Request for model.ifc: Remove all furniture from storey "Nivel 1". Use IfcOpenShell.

First a look at what the model holds.

```python
import ifcopenshell
import ifcopenshell.util.element

model = ifcopenshell.open("model.ifc")
print(model.schema)
storey = next(s for s in model.by_type("IfcBuildingStorey") if s.Name == "Nivel 1")
furniture = [e for e in ifcopenshell.util.element.get_decomposition(storey) if e.is_a("IfcFurnishingElement")]
seen = {}
for e in furniture:
    element_type = ifcopenshell.util.element.get_type(e)
    name = element_type.Name if element_type not in (None, e) else None
    seen[name] = seen.get(name, 0) + 1
for name, count in sorted(seen.items(), key=str):
    print(count, "x", name)
```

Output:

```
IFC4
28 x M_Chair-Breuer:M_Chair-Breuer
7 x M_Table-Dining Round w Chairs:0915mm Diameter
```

```python
import ifcopenshell
import ifcopenshell.api.root
import ifcopenshell.util.element

model = ifcopenshell.open("model.ifc")

storey = next(s for s in model.by_type("IfcBuildingStorey") if s.Name == "Nivel 1")
furniture = [e for e in ifcopenshell.util.element.get_decomposition(storey) if e.is_a("IfcFurnishingElement")]

for e in furniture:
    ifcopenshell.api.root.remove_product(model, product=e)
print(len(furniture), "removed")

model.write("model_updated.ifc")
```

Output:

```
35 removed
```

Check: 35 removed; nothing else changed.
